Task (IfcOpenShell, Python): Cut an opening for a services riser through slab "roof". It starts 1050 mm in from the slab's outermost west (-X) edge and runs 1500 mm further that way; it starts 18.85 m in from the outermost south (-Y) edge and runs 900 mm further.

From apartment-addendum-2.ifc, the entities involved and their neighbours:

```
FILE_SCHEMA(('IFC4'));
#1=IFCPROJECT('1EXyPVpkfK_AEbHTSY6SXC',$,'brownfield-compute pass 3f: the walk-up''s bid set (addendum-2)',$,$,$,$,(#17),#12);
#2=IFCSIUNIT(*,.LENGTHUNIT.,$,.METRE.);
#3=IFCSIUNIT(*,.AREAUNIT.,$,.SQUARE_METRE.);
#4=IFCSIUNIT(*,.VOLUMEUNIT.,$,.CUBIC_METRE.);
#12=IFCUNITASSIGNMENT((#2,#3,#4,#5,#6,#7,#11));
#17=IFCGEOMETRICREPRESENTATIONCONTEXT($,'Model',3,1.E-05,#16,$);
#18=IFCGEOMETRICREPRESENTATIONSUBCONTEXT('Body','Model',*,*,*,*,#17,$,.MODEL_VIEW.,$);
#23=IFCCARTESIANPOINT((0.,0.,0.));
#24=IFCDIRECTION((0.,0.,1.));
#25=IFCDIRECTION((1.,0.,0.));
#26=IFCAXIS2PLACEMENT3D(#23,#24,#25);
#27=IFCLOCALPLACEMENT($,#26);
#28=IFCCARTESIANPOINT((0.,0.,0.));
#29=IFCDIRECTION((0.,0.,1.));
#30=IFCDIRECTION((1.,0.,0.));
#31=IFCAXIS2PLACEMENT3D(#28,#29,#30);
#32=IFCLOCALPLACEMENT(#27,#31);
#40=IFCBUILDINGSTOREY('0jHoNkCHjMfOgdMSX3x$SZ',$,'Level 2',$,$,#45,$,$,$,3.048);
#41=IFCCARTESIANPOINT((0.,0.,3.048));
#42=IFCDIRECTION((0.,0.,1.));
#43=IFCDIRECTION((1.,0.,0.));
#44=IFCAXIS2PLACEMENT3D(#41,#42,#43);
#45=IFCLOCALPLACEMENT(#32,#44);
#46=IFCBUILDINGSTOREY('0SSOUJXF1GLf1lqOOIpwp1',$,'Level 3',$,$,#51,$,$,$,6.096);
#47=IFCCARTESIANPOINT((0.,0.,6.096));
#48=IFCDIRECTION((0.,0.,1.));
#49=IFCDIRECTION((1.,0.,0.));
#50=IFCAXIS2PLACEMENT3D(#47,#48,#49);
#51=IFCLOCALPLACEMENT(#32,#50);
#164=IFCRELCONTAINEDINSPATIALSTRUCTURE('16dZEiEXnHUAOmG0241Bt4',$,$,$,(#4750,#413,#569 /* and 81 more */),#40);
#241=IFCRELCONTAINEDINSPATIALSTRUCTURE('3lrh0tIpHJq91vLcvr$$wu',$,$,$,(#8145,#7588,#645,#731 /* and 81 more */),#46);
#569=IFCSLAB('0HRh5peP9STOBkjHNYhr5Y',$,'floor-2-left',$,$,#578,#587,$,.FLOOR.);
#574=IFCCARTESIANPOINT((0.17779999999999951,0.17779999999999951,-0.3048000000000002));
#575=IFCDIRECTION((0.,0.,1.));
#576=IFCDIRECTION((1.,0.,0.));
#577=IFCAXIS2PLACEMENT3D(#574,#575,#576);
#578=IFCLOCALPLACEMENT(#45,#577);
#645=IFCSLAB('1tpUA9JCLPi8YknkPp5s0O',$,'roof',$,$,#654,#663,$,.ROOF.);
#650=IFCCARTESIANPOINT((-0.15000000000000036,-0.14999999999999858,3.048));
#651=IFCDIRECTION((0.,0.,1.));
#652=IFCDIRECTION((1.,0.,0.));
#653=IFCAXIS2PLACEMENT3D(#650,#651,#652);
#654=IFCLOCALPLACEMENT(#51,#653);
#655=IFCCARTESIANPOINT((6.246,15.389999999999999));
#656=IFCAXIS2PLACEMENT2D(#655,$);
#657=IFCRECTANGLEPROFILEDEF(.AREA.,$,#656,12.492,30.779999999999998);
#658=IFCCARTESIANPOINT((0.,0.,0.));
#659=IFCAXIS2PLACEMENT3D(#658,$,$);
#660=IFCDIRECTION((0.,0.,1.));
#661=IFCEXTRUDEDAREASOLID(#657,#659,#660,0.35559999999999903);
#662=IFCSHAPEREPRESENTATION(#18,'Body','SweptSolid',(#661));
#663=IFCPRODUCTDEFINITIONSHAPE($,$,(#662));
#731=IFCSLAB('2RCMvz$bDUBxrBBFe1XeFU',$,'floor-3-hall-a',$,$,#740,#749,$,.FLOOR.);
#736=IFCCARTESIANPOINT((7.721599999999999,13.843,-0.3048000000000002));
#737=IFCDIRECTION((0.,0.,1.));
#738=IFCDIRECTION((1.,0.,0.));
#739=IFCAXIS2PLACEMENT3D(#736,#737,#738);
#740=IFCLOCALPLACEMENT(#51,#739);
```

```python
import numpy as np
import ifcopenshell
import ifcopenshell.api.feature
import ifcopenshell.api.geometry
import ifcopenshell.api.root
import ifcopenshell.geom
import ifcopenshell.util.placement
import ifcopenshell.util.representation
import ifcopenshell.util.shape
import ifcopenshell.util.unit

model = ifcopenshell.open("apartment-addendum-2.ifc")
unit_scale = ifcopenshell.util.unit.calculate_unit_scale(model)
settings = ifcopenshell.geom.settings()


def volume(element):
    """Net volume in cubic metres, openings subtracted."""
    shape = ifcopenshell.geom.create_shape(settings, element)
    return ifcopenshell.util.shape.get_volume(shape.geometry)


slab = model.by_id(645)
before = volume(slab)

# Extent in the slab's own axes, in metres. The edges named are its -X and -Y sides.
slab_shape = ifcopenshell.geom.create_shape(settings, slab)
vertices = ifcopenshell.util.shape.get_vertices(slab_shape.geometry)
x_min, y_min, bottom = vertices.min(axis=0)
top = vertices[:, 2].max()

opening = ifcopenshell.api.root.create_entity(model, ifc_class="IfcOpeningElement", name="Services riser opening", predefined_type="OPENING")
context = ifcopenshell.util.representation.get_context(model, "Model", "Body", "MODEL_VIEW")
width, depth = 1.5, 0.9
outline = [(0.0, 0.0), (width, 0.0), (width, depth), (0.0, depth), (0.0, 0.0)]
# Overshoot both faces by 50 mm so the cut is clean.
shape = ifcopenshell.api.geometry.add_slab_representation(
    model, context=context, depth=top - bottom + 0.1, polyline=outline
)
ifcopenshell.api.geometry.assign_representation(model, product=opening, representation=shape)

matrix = ifcopenshell.util.placement.get_local_placement(slab.ObjectPlacement)
matrix[:, 3] = matrix @ np.append(np.array([x_min + 1.05, y_min + 18.85, bottom - 0.05]) / unit_scale, 1.0)
ifcopenshell.api.geometry.edit_object_placement(model, product=opening, matrix=matrix, is_si=False)
ifcopenshell.api.feature.add_feature(model, feature=opening, element=slab)

after = volume(slab)

print(f"slab volume {before:.3f} -> {after:.3f} m3")

model.write("apartment-addendum-2-out.ifc")
```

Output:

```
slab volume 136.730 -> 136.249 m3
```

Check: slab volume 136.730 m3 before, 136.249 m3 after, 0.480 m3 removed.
